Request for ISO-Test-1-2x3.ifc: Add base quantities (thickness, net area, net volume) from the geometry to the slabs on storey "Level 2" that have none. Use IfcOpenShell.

First a look at what the model holds.

```python
import ifcopenshell
import ifcopenshell.util.element
import ifcopenshell.util.unit

model = ifcopenshell.open("ISO-Test-1-2x3.ifc")
print(model.schema)
for unit_type in ("LENGTHUNIT", "AREAUNIT", "VOLUMEUNIT"):
    print(unit_type, ifcopenshell.util.unit.calculate_unit_scale(model, unit_type))
storey = next(s for s in model.by_type("IfcBuildingStorey") if s.Name == "Level 2")
slabs = [e for e in ifcopenshell.util.element.get_decomposition(storey) if e.is_a("IfcSlab")]
for e in sorted(slabs, key=lambda e: e.id()):
    print(e.id(), e.is_a(), e.Name, list(ifcopenshell.util.element.get_psets(e, qtos_only=True)), sep=" | ")
```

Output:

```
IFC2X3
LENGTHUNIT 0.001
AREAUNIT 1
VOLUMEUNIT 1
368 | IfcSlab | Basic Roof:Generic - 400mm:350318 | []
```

```python
import ifcopenshell
import ifcopenshell.api.pset
import ifcopenshell.geom
import ifcopenshell.util.element
import ifcopenshell.util.shape
import ifcopenshell.util.unit

model = ifcopenshell.open("ISO-Test-1-2x3.ifc")
unit_scale = ifcopenshell.util.unit.calculate_unit_scale(model)
area_scale = ifcopenshell.util.unit.calculate_unit_scale(model, "AREAUNIT")
volume_scale = ifcopenshell.util.unit.calculate_unit_scale(model, "VOLUMEUNIT")
settings = ifcopenshell.geom.settings()

storey = next(s for s in model.by_type("IfcBuildingStorey") if s.Name == "Level 2")
slabs = [e for e in ifcopenshell.util.element.get_decomposition(storey) if e.is_a("IfcSlab")]

for e in sorted(slabs, key=lambda e: e.id()):
    if ifcopenshell.util.element.get_psets(e, qtos_only=True, should_inherit=False):
        continue
    # Geometry comes back in metres, in the element's own axes.
    shape = ifcopenshell.geom.create_shape(settings, e)
    values = {
        "Width": ifcopenshell.util.shape.get_z(shape.geometry) / unit_scale,
        "NetArea": ifcopenshell.util.shape.get_footprint_area(shape.geometry) / area_scale,
        "NetVolume": ifcopenshell.util.shape.get_volume(shape.geometry) / volume_scale,
    }
    qto = ifcopenshell.api.pset.add_qto(model, product=e, name="BaseQuantities")
    ifcopenshell.api.pset.edit_qto(model, qto=qto, properties=values)
    print(e.id(), {k: round(v, 3) for k, v in values.items()})

model.write("ISO-Test-1-2x3_edited.ifc")
```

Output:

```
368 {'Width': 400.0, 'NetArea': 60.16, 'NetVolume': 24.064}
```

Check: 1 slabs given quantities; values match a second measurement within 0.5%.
